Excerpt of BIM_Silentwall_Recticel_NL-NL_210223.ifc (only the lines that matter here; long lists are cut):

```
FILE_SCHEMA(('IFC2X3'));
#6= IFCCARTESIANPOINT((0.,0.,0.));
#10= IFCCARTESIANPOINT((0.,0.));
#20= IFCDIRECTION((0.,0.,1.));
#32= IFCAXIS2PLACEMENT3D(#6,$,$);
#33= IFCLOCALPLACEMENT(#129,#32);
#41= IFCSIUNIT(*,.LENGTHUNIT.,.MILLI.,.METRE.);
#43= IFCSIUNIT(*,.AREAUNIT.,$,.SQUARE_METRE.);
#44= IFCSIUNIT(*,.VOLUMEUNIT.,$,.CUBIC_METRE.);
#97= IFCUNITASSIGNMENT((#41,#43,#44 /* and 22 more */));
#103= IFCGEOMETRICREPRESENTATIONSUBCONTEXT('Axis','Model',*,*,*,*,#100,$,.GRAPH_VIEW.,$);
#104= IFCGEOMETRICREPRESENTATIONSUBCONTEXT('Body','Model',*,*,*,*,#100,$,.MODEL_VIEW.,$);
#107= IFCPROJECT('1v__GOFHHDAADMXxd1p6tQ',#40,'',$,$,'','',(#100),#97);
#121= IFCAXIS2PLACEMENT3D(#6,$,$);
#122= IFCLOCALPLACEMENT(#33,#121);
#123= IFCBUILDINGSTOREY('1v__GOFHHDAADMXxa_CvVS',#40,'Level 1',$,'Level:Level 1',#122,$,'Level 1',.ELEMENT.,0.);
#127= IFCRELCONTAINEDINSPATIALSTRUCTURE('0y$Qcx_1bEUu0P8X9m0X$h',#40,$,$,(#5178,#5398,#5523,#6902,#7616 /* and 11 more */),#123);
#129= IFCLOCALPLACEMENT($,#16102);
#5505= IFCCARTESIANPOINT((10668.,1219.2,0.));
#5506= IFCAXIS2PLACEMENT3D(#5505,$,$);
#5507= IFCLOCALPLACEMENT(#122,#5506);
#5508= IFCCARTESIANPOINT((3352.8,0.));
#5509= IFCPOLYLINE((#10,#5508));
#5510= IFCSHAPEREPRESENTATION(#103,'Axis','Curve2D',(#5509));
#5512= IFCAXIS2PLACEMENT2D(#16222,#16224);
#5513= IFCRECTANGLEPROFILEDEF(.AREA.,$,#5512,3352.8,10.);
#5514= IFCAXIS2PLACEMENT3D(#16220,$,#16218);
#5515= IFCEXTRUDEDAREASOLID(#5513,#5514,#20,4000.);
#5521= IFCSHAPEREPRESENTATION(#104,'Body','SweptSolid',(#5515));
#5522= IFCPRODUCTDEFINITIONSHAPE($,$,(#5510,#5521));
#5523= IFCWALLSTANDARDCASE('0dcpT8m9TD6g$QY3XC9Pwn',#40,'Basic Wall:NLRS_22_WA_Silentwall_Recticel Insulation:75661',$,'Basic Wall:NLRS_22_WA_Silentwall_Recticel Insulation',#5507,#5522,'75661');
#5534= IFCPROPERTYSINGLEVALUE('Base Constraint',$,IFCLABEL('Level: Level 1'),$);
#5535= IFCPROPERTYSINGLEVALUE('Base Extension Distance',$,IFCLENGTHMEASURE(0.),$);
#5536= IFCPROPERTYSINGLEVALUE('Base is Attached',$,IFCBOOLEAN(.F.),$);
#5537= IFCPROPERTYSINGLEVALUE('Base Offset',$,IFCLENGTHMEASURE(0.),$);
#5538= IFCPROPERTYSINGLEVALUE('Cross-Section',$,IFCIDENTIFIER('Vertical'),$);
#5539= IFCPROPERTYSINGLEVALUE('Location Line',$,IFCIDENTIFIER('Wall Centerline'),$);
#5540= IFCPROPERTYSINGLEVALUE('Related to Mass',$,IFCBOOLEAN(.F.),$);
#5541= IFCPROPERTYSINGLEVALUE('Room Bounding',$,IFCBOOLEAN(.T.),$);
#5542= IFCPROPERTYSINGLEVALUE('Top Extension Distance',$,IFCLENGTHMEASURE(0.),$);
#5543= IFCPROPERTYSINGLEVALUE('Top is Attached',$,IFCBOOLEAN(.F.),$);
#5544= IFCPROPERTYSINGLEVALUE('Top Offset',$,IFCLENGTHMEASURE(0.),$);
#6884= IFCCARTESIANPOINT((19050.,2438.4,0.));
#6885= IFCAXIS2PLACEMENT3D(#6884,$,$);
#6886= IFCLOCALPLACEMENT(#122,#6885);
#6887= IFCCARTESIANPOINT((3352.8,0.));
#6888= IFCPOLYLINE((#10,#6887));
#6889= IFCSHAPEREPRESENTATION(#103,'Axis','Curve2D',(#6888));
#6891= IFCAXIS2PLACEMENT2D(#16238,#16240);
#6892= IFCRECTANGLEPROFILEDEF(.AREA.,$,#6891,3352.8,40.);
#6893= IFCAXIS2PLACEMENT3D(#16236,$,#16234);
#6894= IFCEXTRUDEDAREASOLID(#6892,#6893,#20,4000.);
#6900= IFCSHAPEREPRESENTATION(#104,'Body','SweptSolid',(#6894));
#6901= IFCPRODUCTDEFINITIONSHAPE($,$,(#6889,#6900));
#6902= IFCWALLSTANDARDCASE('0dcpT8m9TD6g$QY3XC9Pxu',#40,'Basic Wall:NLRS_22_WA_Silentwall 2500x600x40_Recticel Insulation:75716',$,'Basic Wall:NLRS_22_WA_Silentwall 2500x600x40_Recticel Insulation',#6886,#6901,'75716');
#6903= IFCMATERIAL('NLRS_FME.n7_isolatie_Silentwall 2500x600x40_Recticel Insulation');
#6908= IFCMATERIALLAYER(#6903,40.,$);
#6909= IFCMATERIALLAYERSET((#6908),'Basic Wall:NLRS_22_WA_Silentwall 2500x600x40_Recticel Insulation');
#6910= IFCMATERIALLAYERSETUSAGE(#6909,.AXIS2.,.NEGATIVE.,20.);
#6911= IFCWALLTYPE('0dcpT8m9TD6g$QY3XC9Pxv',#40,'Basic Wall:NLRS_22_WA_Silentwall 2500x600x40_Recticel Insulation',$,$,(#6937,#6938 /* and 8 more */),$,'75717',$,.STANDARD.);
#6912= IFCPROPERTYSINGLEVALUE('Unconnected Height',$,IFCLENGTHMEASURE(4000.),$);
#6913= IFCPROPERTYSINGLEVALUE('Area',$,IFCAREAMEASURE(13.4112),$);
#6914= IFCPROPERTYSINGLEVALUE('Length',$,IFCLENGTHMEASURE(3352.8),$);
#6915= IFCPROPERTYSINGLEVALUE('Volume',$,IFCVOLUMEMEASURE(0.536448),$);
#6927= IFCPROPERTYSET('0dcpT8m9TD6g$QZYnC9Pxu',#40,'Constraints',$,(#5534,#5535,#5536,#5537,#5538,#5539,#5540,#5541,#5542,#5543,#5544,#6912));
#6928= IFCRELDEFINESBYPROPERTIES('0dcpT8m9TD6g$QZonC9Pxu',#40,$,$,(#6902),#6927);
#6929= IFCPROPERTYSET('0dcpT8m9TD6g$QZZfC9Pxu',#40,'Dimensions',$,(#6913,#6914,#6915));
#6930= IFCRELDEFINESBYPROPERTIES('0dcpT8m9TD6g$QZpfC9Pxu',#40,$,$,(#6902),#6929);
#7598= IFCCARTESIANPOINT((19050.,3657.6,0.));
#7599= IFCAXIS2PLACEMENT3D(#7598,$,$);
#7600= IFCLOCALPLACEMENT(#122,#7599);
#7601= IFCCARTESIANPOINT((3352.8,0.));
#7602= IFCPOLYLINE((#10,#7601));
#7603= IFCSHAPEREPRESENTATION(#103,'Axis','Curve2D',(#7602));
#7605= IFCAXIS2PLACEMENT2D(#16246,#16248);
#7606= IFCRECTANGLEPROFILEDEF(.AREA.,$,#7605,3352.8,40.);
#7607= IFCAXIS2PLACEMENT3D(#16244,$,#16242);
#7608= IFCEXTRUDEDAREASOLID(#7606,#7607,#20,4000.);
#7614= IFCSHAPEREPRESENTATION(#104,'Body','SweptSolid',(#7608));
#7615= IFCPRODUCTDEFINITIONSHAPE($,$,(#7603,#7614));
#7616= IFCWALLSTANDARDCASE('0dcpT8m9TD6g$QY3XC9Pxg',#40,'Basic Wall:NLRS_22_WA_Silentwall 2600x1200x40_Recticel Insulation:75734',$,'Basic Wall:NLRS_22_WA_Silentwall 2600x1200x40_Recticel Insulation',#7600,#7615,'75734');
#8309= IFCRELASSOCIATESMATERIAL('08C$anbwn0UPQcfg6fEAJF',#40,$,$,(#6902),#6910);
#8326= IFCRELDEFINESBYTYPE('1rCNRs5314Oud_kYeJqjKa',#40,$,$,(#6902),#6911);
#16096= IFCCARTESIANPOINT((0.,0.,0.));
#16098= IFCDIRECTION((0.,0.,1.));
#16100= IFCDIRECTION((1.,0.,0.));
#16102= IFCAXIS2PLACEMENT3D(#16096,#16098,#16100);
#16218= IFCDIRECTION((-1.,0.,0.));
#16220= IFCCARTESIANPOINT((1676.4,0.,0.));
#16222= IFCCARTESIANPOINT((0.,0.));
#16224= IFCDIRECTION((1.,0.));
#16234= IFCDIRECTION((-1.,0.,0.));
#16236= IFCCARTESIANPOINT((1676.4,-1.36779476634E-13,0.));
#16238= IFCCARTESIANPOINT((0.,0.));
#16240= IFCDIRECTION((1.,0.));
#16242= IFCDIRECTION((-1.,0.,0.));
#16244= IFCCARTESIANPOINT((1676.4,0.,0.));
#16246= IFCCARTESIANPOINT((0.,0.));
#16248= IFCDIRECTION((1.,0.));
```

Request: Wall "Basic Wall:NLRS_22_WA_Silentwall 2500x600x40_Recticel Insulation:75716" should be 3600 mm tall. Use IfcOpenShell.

```python
import ifcopenshell
import ifcopenshell.api.pset
import ifcopenshell.geom
import ifcopenshell.util.element
import ifcopenshell.util.representation
import ifcopenshell.util.shape
import ifcopenshell.util.unit

model = ifcopenshell.open("BIM_Silentwall_Recticel_NL-NL_210223.ifc")
area_scale = ifcopenshell.util.unit.calculate_unit_scale(model, "AREAUNIT")
volume_scale = ifcopenshell.util.unit.calculate_unit_scale(model, "VOLUMEUNIT")
settings = ifcopenshell.geom.settings()


def volume(element):
    """Net volume in cubic metres, openings subtracted."""
    shape = ifcopenshell.geom.create_shape(settings, element)
    return ifcopenshell.util.shape.get_volume(shape.geometry)


wall = model.by_guid("0dcpT8m9TD6g$QY3XC9Pxu")
before = volume(wall)

body = ifcopenshell.util.representation.get_representation(wall, "Model", "Body")
solid = body.Items[0]
old_height = solid.Depth
solid.Depth = 3600.0
after = volume(wall)
thickness = 0.04  # wall thickness in metres

# Update the stored height, areas and volumes.
pset = model.by_id(ifcopenshell.util.element.get_pset(wall, "Constraints", should_inherit=False)["id"])
ifcopenshell.api.pset.edit_pset(model, pset=pset, properties={
    "Unconnected Height": model.create_entity("IfcLengthMeasure", solid.Depth),
})
pset = model.by_id(ifcopenshell.util.element.get_pset(wall, "Dimensions", should_inherit=False)["id"])
ifcopenshell.api.pset.edit_pset(model, pset=pset, properties={
    "Area": model.create_entity("IfcAreaMeasure", after / thickness / area_scale),
    "Volume": model.create_entity("IfcVolumeMeasure", after / volume_scale),
})

print(f"height {old_height:g} -> {solid.Depth:g}, volume {before:.3f} -> {after:.3f} m3")

model.write("BIM_Silentwall_Recticel_NL-NL_210223_rev.ifc")
```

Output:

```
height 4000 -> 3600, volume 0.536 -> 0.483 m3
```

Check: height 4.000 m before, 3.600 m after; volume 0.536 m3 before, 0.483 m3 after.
